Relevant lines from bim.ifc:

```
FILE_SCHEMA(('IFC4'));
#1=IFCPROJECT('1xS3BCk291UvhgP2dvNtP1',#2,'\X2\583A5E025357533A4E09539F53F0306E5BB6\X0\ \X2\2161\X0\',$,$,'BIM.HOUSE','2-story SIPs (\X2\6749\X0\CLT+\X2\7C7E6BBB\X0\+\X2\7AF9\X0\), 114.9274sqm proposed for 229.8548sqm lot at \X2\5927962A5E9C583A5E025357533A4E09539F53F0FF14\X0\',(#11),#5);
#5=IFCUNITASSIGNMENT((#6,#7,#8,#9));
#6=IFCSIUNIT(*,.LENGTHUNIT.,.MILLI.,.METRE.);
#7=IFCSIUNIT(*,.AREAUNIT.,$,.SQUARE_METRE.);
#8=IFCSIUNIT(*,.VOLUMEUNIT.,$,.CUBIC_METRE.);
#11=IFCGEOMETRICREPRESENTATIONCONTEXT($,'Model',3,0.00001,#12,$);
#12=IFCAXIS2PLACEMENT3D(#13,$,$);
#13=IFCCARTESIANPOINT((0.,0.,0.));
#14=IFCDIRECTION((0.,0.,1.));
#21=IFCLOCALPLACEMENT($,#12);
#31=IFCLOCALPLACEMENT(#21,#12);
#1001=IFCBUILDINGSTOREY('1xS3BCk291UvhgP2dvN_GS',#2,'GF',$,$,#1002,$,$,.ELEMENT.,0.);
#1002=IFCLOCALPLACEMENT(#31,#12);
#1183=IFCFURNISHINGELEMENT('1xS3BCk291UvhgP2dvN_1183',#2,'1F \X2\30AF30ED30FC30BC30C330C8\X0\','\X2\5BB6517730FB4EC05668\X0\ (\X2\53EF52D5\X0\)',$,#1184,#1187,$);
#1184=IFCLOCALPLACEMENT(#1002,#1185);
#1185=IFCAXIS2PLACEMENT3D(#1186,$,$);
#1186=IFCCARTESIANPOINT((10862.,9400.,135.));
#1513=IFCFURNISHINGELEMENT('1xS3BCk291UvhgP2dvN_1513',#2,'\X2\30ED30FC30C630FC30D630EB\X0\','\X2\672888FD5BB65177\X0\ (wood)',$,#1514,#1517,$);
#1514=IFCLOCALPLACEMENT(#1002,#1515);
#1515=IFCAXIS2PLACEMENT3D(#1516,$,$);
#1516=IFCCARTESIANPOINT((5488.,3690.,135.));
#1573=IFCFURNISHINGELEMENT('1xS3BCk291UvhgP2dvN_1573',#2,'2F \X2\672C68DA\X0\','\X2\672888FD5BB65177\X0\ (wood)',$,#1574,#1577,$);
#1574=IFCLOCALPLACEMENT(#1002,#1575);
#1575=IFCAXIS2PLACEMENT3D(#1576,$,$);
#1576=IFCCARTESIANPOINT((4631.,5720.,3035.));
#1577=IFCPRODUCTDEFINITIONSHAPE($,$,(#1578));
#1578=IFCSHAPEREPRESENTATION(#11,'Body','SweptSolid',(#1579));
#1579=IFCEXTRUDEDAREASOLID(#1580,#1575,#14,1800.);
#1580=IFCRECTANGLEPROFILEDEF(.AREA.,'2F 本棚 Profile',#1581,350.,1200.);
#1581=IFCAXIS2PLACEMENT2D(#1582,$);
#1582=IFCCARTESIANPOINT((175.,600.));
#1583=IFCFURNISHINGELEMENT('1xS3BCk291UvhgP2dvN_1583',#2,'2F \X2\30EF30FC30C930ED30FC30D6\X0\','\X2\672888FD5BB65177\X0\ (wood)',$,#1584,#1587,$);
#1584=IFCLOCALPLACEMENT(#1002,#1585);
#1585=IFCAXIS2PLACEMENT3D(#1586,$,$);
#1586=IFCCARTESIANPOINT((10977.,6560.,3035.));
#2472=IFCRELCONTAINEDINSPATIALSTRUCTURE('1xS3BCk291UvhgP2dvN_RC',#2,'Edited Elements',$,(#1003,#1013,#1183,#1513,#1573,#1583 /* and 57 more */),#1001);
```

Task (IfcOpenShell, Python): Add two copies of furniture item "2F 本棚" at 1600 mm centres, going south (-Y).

```python
import numpy as np
import ifcopenshell
import ifcopenshell.api.geometry
import ifcopenshell.api.root
import ifcopenshell.util.element
import ifcopenshell.util.placement
import ifcopenshell.util.unit

model = ifcopenshell.open("bim.ifc")
unit_scale = ifcopenshell.util.unit.calculate_unit_scale(model)


def reuse_history(source, copy):
    """copy_class also copies each property set's owner history, people and application; keep the originals."""
    for rel in copy.IsDefinedBy:
        if rel.is_a("IfcRelDefinesByProperties") and (history := rel.RelatingPropertyDefinition.OwnerHistory):
            rel.RelatingPropertyDefinition.OwnerHistory = source.OwnerHistory
            ifcopenshell.util.element.remove_deep2(model, history)


source = model.by_guid("1xS3BCk291UvhgP2dvN_1573")
base = ifcopenshell.util.placement.get_local_placement(source.ObjectPlacement)
step = np.array([0.0, -1.0, 0.0]) * 1.6 / unit_scale

for i in range(1, 3):
    copy = ifcopenshell.api.root.copy_class(model, product=source)
    copy.Representation = ifcopenshell.util.element.copy_deep(
        model, source.Representation, exclude=["IfcGeometricRepresentationContext", "IfcRepresentationMap"]
    )
    reuse_history(source, copy)
    matrix = base.copy()
    matrix[:3, 3] += i * step
    print("added at", matrix[:3, 3].round(3) + 0.0)
    ifcopenshell.api.geometry.edit_object_placement(model, product=copy, matrix=matrix, is_si=False)

model.write("bim_rev.ifc")
```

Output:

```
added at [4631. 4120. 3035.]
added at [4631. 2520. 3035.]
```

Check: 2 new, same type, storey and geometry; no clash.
